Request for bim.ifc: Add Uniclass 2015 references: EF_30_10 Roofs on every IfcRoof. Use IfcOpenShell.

First a look at what the model holds.

```python
import ifcopenshell

model = ifcopenshell.open("bim.ifc")
print(model.schema)
print("classifications:", [c.Name for c in model.by_type("IfcClassification")])
for ifc_class in ("IfcDoor", "IfcRoof", "IfcStair", "IfcWall", "IfcWindow"):
    print(ifc_class, len(model.by_type(ifc_class)))
```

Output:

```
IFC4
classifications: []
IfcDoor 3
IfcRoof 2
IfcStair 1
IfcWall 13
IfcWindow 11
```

```python
import ifcopenshell
import ifcopenshell.api.classification

model = ifcopenshell.open("bim.ifc")

system = ifcopenshell.api.classification.add_classification(model, classification="Uniclass 2015")

codes = {
    "IfcRoof": ("EF_30_10", "Roofs"),
}
for ifc_class, (code, name) in codes.items():
    products = model.by_type(ifc_class)
    ifcopenshell.api.classification.add_reference(
        model, products=products, classification=system, identification=code, name=name
    )
    print(code, len(products))

model.write("bim_edited.ifc")
```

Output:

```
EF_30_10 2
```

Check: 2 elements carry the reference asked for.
